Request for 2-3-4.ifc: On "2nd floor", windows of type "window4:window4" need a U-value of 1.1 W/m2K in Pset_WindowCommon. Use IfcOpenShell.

First a look at what the model holds.

```python
import ifcopenshell
import ifcopenshell.util.element

model = ifcopenshell.open("2-3-4.ifc")
print(model.schema)
storey = next(s for s in model.by_type("IfcBuildingStorey") if s.Name == "2nd floor")
windows = [e for e in ifcopenshell.util.element.get_decomposition(storey) if e.is_a("IfcWindow")]
seen = {}
for e in windows:
    element_type = ifcopenshell.util.element.get_type(e)
    key = (element_type.Name if element_type != e and element_type else None, ifcopenshell.util.element.get_pset(e, "Pset_WindowCommon", "ThermalTransmittance"))
    seen[key] = seen.get(key, 0) + 1
for (name, value), count in sorted(seen.items(), key=str):
    print(count, "x", name, "|", value)
```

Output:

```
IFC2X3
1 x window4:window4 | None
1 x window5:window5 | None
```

```python
import ifcopenshell
import ifcopenshell.api.pset
import ifcopenshell.util.element

model = ifcopenshell.open("2-3-4.ifc")

storey = next(s for s in model.by_type("IfcBuildingStorey") if s.Name == "2nd floor")
windows = [e for e in ifcopenshell.util.element.get_decomposition(storey) if e.is_a("IfcWindow")]

count = 0
for e in windows:
    element_type = ifcopenshell.util.element.get_type(e)
    if element_type in (None, e) or element_type.Name != "window4:window4":
        continue
    # add_pset returns the element's existing set when there is one.
    pset = ifcopenshell.api.pset.add_pset(model, product=e, name="Pset_WindowCommon")
    ifcopenshell.api.pset.edit_pset(model, pset=pset, properties={"ThermalTransmittance": 1.1})
    count += 1

print(count, "windows updated")

model.write("2-3-4_edited.ifc")
```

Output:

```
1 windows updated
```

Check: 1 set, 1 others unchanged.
